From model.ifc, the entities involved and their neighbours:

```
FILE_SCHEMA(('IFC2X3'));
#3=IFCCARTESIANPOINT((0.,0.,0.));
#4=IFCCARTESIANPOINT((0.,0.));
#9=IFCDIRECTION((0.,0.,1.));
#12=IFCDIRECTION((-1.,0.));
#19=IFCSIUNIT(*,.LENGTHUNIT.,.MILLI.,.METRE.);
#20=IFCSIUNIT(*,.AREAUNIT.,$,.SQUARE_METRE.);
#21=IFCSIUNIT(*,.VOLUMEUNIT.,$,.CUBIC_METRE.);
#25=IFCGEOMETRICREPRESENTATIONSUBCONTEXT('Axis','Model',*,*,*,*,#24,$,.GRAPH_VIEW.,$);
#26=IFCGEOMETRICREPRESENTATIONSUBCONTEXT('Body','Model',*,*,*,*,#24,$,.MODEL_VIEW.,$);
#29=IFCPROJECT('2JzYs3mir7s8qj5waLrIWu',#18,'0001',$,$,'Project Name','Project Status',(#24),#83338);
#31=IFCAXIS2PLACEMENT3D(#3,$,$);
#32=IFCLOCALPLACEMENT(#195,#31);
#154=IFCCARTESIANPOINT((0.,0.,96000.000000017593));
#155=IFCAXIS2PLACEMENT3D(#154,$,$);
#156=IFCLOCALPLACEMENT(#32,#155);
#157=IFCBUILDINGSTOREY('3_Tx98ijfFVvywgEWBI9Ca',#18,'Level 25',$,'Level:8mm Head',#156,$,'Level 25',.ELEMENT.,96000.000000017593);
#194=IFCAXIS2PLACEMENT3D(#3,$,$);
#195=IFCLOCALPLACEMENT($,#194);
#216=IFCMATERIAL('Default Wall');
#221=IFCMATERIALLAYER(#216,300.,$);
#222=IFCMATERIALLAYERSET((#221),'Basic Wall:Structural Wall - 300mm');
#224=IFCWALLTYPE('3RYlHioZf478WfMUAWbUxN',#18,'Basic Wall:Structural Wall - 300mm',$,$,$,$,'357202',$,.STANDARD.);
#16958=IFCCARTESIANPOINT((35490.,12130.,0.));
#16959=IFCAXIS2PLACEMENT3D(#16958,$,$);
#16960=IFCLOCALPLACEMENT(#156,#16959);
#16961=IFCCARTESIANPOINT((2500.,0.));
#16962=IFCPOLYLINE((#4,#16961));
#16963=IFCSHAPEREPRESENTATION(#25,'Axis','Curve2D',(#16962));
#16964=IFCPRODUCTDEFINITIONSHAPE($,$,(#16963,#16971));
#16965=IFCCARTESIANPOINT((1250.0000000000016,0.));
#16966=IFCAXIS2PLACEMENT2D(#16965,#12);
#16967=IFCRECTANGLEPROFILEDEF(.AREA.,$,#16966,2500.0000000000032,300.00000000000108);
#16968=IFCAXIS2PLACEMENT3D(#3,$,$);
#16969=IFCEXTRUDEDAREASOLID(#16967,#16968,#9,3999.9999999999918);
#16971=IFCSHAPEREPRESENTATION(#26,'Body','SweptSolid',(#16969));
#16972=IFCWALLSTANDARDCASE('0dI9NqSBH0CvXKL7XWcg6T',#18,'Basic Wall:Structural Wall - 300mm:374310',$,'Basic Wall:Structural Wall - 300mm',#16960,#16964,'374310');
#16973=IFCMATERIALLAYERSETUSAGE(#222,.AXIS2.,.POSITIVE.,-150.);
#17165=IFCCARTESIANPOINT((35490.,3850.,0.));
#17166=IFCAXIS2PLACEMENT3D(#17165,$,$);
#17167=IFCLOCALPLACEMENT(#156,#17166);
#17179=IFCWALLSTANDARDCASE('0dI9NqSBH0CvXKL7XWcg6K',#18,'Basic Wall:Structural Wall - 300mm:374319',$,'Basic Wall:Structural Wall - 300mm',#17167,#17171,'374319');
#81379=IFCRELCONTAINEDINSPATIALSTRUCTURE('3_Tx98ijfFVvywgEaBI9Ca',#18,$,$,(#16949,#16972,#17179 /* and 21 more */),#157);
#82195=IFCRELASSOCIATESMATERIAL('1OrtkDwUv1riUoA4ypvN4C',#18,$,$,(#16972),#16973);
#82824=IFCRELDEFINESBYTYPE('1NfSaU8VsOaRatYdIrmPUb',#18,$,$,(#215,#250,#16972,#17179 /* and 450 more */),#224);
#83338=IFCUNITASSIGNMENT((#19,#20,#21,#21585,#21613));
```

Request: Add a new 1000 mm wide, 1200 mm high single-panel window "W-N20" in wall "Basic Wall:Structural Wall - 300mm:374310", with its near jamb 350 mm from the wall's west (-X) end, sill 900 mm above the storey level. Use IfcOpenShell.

```python
import numpy as np
import ifcopenshell
import ifcopenshell.api.feature
import ifcopenshell.api.geometry
import ifcopenshell.api.root
import ifcopenshell.api.spatial
import ifcopenshell.api.type
import ifcopenshell.geom
import ifcopenshell.util.element
import ifcopenshell.util.placement
import ifcopenshell.util.representation
import ifcopenshell.util.shape
import ifcopenshell.util.unit

model = ifcopenshell.open("model.ifc")
unit_scale = ifcopenshell.util.unit.calculate_unit_scale(model)
settings = ifcopenshell.geom.settings()


def volume(element):
    """Net volume in cubic metres, openings subtracted."""
    shape = ifcopenshell.geom.create_shape(settings, element)
    return ifcopenshell.util.shape.get_volume(shape.geometry)


wall = model.by_guid("0dI9NqSBH0CvXKL7XWcg6T")
storey = ifcopenshell.util.element.get_container(wall, ifc_class="IfcBuildingStorey")
context = ifcopenshell.util.representation.get_context(model, "Model", "Body", "MODEL_VIEW")
before = volume(wall)

width, height, from_end, sill = 1, 1.2, 0.35, 0.9  # metres

# The wall runs along its own X axis, and the end named is its -X end.
wall_shape = ifcopenshell.geom.create_shape(settings, wall)
x, y, z = ifcopenshell.util.shape.get_vertices(wall_shape.geometry).T
start = x.min() + from_end
face, thickness = float(y.min()), float(y.max() - y.min())
wall_matrix = ifcopenshell.util.placement.get_local_placement(wall.ObjectPlacement)
level = ifcopenshell.util.placement.get_local_placement(storey.ObjectPlacement)[2, 3]


def in_wall(x, y):
    """Placement at x, y metres in the wall's axes, at sill height."""
    matrix = wall_matrix.copy()
    matrix[:, 3] = wall_matrix @ np.array([x / unit_scale, y / unit_scale, 0.0, 1.0])
    matrix[2, 3] = level + sill / unit_scale
    return matrix


# Opening: a box that overshoots both wall faces by 50 mm.
opening = ifcopenshell.api.root.create_entity(model, ifc_class="IfcOpeningElement")
box = ifcopenshell.api.geometry.add_wall_representation(
    model, context=context, length=width, height=height, thickness=thickness + 0.1
)
ifcopenshell.api.geometry.assign_representation(model, product=opening, representation=box)
ifcopenshell.api.geometry.edit_object_placement(model, product=opening, matrix=in_wall(start, face - 0.05), is_si=False)
ifcopenshell.api.feature.add_feature(model, feature=opening, element=wall)

window = ifcopenshell.api.root.create_entity(model, ifc_class="IfcWindow", name="W-N20")
window.OverallWidth, window.OverallHeight = width / unit_scale, height / unit_scale
body = ifcopenshell.api.geometry.add_window_representation(
    model,
    context=context,
    overall_width=window.OverallWidth,
    overall_height=window.OverallHeight,
    partition_type="SINGLE_PANEL",
)
ifcopenshell.api.geometry.assign_representation(model, product=window, representation=body)
ifcopenshell.api.spatial.assign_container(model, products=[window], relating_structure=storey)
fills = ifcopenshell.api.feature.add_filling(model, opening=opening, element=window)
fills.OwnerHistory = window.OwnerHistory  # required in IFC2X3

# IFC2X3 keeps the operation on the window style.
style = ifcopenshell.api.root.create_entity(model, ifc_class="IfcWindowStyle", name="W-N20")
style.OperationType, style.ConstructionType = "SINGLE_PANEL", "NOTDEFINED"
style.ParameterTakesPrecedence = style.Sizeable = False
ifcopenshell.api.type.assign_type(model, related_objects=[window], relating_type=style)

# Centre the window in the wall's thickness.
ifcopenshell.api.geometry.edit_object_placement(model, product=window, matrix=in_wall(start, face), is_si=False)
window_shape = ifcopenshell.geom.create_shape(settings, window)
depth = ifcopenshell.util.shape.get_vertices(window_shape.geometry)[:, 1]
offset = face + thickness / 2 - (depth.min() + depth.max()) / 2
ifcopenshell.api.geometry.edit_object_placement(model, product=window, matrix=in_wall(start, offset), is_si=False)

after = volume(wall)

print(f"wall volume {before:.3f} -> {after:.3f} m3")

model.write("model_edited.ifc")
```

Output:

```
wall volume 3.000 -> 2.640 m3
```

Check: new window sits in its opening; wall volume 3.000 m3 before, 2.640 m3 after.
